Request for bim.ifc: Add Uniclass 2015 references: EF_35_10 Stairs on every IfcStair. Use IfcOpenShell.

First a look at what the model holds.

```python
import ifcopenshell

model = ifcopenshell.open("bim.ifc")
print(model.schema)
print("classifications:", [c.Name for c in model.by_type("IfcClassification")])
for ifc_class in ("IfcDoor", "IfcRoof", "IfcStair", "IfcWall", "IfcWindow"):
    print(ifc_class, len(model.by_type(ifc_class)))
```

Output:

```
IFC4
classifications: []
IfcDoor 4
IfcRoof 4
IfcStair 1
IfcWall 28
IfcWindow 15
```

```python
import ifcopenshell
import ifcopenshell.api.classification

model = ifcopenshell.open("bim.ifc")

system = ifcopenshell.api.classification.add_classification(model, classification="Uniclass 2015")

codes = {
    "IfcStair": ("EF_35_10", "Stairs"),
}
for ifc_class, (code, name) in codes.items():
    products = model.by_type(ifc_class)
    ifcopenshell.api.classification.add_reference(
        model, products=products, classification=system, identification=code, name=name
    )
    print(code, len(products))

model.write("bim_rev.ifc")
```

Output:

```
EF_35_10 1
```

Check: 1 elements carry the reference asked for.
